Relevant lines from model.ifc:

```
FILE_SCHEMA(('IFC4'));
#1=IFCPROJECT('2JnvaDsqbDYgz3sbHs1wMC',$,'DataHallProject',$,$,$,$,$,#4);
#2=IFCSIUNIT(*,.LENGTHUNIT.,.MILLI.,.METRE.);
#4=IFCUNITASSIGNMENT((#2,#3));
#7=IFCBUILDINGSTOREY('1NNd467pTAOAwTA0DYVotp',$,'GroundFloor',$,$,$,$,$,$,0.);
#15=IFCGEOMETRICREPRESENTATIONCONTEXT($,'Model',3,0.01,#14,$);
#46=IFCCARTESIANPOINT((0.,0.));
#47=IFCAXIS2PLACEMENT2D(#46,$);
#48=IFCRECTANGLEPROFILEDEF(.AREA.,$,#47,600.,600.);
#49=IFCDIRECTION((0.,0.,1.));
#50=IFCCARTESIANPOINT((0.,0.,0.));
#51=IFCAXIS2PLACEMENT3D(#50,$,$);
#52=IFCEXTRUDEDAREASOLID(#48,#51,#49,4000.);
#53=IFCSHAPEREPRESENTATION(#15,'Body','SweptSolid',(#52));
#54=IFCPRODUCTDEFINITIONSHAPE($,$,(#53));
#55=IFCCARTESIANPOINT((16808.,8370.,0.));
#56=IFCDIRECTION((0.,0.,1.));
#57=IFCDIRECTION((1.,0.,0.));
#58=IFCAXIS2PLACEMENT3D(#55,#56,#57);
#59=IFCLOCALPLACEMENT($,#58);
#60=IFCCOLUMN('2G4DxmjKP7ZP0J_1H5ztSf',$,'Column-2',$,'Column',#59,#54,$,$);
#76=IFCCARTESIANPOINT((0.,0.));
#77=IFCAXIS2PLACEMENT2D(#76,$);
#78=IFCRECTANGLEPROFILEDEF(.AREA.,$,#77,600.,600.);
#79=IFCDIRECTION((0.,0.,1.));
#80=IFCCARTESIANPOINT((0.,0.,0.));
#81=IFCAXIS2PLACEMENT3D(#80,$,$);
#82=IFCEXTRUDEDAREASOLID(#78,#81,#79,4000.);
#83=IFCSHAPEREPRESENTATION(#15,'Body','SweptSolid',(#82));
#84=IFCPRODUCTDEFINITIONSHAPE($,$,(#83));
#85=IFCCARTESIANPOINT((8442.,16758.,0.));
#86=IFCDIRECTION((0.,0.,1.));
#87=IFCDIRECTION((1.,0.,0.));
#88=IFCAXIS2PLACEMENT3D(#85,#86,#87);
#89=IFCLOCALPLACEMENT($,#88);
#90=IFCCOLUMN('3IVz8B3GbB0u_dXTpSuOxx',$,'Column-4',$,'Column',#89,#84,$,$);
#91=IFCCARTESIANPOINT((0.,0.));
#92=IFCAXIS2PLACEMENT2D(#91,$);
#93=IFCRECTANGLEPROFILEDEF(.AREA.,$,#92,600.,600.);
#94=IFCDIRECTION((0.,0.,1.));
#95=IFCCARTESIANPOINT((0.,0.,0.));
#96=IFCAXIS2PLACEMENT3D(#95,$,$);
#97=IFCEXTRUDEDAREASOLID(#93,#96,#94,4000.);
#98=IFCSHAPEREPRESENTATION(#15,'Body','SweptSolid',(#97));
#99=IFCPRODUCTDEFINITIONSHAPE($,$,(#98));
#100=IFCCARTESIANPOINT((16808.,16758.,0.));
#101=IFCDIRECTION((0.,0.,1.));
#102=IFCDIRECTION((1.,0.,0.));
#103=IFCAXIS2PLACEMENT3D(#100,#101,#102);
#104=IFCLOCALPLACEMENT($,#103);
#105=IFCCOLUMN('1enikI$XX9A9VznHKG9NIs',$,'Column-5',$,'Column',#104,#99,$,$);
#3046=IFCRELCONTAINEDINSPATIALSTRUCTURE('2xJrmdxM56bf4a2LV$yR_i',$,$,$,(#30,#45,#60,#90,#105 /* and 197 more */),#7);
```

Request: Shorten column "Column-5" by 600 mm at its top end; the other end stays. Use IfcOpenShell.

```python
import ifcopenshell
import ifcopenshell.util.unit

model = ifcopenshell.open("model.ifc")
unit_scale = ifcopenshell.util.unit.calculate_unit_scale(model)

member = model.by_id(105)
change = -0.6 / unit_scale

# The extrusion runs towards the end named, so only its depth changes.
body = next(r for r in member.Representation.Representations if r.RepresentationIdentifier == "Body")
solid = body.Items[0]
old_length = solid.Depth
solid.Depth += change

print(f"length {old_length:g} -> {solid.Depth:g}")

model.write("model_rev.ifc")
```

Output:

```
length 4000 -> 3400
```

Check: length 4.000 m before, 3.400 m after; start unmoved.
